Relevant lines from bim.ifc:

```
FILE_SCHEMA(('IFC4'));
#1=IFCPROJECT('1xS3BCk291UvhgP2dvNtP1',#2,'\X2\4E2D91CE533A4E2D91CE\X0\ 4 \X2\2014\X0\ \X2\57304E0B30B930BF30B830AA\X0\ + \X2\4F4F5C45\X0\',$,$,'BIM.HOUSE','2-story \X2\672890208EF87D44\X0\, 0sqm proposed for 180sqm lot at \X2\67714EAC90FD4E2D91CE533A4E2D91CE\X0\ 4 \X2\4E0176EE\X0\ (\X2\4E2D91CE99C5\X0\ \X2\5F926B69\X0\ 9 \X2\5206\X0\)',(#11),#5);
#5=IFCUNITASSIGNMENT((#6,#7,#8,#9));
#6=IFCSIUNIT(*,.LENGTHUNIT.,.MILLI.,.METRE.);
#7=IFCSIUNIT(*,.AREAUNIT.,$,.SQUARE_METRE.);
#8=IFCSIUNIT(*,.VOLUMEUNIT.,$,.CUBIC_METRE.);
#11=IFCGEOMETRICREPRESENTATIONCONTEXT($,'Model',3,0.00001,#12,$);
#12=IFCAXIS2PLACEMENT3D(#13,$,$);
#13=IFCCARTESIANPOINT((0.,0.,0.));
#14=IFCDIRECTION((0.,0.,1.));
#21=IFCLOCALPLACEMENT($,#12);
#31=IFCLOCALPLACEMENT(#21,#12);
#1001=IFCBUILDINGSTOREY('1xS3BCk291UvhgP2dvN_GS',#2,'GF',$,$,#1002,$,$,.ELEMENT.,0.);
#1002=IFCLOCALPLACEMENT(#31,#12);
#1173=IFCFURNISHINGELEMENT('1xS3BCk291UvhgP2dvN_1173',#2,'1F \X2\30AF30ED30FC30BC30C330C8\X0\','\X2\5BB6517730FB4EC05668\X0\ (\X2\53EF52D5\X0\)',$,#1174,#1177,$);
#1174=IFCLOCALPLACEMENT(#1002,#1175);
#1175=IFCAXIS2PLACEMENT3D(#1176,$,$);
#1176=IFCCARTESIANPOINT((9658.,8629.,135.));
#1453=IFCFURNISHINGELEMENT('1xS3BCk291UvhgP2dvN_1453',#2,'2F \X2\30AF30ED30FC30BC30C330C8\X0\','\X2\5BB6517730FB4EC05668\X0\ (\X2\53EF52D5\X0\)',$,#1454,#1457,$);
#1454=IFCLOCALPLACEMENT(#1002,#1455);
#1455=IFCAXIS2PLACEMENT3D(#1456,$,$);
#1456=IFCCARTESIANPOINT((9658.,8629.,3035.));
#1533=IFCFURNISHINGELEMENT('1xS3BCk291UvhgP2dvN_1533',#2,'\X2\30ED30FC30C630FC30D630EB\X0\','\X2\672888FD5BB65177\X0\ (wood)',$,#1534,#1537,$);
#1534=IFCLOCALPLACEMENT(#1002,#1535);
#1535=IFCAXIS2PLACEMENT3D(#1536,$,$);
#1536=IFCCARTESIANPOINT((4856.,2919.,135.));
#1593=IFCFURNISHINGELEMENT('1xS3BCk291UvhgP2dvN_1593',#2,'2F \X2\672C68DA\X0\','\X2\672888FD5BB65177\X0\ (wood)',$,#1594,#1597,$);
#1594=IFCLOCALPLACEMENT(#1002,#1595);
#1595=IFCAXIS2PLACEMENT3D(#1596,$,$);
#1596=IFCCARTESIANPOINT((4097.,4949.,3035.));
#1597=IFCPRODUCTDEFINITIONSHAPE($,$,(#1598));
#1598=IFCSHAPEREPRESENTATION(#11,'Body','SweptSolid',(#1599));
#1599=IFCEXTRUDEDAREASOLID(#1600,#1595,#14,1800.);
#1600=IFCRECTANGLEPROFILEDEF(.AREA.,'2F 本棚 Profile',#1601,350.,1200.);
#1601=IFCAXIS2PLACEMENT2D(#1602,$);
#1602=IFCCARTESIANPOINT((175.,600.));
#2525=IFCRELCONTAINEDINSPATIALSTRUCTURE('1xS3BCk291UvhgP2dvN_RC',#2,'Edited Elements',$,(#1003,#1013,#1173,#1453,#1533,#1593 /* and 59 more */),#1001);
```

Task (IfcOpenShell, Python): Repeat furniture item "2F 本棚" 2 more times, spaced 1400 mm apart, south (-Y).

```python
import numpy as np
import ifcopenshell
import ifcopenshell.api.geometry
import ifcopenshell.api.root
import ifcopenshell.util.element
import ifcopenshell.util.placement

model = ifcopenshell.open("bim.ifc")


def reuse_history(source, copy):
    """copy_class also copies each property set's owner history, people and application; keep the originals."""
    for rel in copy.IsDefinedBy:
        if rel.is_a("IfcRelDefinesByProperties") and (history := rel.RelatingPropertyDefinition.OwnerHistory):
            rel.RelatingPropertyDefinition.OwnerHistory = source.OwnerHistory
            ifcopenshell.util.element.remove_deep2(model, history)


source = model.by_guid("1xS3BCk291UvhgP2dvN_1593")
base = ifcopenshell.util.placement.get_local_placement(source.ObjectPlacement)
step = np.array([0.0, -1.0, 0.0]) * 1400.0

for i in range(1, 3):
    copy = ifcopenshell.api.root.copy_class(model, product=source)
    copy.Representation = ifcopenshell.util.element.copy_deep(
        model, source.Representation, exclude=["IfcGeometricRepresentationContext", "IfcRepresentationMap"]
    )
    reuse_history(source, copy)
    matrix = base.copy()
    matrix[:3, 3] += i * step
    print("added at", matrix[:3, 3].round(3) + 0.0)
    ifcopenshell.api.geometry.edit_object_placement(model, product=copy, matrix=matrix, is_si=False)

model.write("bim_rev.ifc")
```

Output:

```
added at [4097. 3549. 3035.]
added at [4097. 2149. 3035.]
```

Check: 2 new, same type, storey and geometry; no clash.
